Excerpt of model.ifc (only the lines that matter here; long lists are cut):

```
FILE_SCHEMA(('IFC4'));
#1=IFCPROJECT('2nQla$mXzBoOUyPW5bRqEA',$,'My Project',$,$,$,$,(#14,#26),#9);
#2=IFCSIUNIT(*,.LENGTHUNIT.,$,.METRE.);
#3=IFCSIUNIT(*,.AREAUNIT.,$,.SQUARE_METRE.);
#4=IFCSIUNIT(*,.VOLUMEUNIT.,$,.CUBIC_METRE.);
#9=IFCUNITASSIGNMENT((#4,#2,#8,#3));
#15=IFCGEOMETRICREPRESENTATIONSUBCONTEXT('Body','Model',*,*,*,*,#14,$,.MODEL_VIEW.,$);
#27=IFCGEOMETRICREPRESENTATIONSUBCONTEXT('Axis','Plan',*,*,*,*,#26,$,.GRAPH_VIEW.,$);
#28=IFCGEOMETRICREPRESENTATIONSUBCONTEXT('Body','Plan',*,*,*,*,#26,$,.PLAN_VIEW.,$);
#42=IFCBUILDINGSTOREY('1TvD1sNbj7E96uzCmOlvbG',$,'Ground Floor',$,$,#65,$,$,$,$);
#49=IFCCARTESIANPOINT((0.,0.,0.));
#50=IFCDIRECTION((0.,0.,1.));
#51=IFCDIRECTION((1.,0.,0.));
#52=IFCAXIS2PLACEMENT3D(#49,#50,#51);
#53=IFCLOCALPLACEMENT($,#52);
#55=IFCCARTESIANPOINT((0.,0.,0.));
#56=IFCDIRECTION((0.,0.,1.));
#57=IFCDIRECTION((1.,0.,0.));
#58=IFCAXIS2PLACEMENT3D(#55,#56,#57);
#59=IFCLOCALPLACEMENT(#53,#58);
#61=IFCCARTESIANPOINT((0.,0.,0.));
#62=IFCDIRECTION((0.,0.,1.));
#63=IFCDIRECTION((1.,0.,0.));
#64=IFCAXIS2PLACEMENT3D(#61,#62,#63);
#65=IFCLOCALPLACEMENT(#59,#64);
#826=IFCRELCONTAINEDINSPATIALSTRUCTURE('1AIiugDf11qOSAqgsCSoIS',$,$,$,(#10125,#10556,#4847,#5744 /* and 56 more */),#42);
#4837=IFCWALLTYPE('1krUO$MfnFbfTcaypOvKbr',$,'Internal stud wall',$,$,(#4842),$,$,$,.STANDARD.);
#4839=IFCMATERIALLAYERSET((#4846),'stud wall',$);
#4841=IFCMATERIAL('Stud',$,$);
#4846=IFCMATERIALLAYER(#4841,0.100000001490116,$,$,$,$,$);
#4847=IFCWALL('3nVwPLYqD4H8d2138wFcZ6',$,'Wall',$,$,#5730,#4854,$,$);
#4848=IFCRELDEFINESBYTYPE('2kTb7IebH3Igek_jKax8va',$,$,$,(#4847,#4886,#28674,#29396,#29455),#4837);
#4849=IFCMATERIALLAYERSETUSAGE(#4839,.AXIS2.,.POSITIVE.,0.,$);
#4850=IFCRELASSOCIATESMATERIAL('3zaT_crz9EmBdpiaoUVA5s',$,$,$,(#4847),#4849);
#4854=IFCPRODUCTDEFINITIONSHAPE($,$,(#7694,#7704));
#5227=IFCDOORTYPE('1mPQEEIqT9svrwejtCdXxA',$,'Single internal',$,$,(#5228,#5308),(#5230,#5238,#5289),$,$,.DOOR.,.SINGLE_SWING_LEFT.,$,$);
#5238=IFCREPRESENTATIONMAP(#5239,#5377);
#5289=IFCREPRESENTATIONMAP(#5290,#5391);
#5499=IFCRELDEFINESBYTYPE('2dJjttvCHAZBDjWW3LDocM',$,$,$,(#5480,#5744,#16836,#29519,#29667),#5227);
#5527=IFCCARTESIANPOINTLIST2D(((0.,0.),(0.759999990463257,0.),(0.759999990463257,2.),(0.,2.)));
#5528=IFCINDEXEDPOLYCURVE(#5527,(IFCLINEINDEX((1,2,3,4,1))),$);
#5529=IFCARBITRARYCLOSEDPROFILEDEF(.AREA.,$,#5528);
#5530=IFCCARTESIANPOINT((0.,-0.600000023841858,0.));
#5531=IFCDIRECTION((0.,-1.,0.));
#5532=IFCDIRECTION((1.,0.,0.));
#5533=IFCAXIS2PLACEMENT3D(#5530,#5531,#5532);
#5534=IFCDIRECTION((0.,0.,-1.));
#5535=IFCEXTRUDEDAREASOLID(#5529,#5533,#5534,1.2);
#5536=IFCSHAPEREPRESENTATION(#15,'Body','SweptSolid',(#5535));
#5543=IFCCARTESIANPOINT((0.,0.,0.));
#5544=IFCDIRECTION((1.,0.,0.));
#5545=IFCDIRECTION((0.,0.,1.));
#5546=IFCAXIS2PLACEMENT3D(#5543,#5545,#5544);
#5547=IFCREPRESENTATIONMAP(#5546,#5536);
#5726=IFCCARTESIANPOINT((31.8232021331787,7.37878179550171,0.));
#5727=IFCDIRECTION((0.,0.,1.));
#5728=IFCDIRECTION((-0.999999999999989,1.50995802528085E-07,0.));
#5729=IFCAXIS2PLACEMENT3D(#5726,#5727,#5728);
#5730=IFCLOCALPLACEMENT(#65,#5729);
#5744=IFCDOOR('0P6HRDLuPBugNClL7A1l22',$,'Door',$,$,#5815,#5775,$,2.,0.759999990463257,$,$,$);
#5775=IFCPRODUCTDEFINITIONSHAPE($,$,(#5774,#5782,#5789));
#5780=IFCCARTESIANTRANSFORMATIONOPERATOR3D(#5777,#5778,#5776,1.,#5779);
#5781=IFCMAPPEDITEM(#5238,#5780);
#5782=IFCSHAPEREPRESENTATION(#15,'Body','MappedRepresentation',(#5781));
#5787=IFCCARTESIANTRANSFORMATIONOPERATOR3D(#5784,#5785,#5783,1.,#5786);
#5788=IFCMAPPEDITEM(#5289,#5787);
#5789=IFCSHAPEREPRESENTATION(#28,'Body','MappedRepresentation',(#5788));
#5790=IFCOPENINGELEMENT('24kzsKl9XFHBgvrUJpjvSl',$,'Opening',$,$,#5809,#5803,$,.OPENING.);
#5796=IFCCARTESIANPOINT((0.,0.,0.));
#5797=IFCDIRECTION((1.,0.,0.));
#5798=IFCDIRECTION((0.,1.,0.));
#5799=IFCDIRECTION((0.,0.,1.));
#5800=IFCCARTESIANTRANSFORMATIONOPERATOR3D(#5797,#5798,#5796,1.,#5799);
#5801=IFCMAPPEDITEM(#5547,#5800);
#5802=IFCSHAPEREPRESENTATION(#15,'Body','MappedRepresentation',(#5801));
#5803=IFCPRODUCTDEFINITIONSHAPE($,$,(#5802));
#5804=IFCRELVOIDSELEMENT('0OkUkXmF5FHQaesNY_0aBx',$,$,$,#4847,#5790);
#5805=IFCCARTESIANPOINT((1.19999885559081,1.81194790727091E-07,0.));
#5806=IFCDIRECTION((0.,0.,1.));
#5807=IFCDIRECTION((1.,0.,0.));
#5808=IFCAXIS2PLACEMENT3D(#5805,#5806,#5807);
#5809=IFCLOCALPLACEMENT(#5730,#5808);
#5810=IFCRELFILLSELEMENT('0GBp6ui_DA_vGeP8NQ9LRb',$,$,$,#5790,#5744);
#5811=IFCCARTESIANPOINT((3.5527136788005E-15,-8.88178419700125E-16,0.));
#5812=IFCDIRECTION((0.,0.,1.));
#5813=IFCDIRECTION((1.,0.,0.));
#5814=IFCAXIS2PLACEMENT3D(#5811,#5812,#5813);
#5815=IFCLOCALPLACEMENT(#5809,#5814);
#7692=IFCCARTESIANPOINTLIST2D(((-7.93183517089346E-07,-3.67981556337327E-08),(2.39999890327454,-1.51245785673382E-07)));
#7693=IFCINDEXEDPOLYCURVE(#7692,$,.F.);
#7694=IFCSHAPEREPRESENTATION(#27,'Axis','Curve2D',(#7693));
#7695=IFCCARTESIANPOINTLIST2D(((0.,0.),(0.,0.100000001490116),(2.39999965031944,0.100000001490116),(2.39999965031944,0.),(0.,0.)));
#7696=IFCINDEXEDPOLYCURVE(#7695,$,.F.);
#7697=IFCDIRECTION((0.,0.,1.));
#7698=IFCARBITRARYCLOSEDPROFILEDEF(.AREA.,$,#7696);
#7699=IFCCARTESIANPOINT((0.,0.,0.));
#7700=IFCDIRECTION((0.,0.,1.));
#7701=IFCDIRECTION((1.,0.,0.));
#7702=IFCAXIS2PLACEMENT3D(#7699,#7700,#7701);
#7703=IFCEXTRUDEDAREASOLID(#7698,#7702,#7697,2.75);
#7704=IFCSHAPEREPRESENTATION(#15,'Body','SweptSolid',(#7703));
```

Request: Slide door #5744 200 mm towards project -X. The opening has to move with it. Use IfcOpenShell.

```python
import ifcopenshell
import ifcopenshell.api.geometry
import ifcopenshell.util.placement
import ifcopenshell.util.unit

model = ifcopenshell.open("model.ifc")
unit_scale = ifcopenshell.util.unit.calculate_unit_scale(model)

door = model.by_guid("0P6HRDLuPBugNClL7A1l22")
opening = door.FillsVoids[0].RelatingOpeningElement
wall = opening.VoidsElements[0].RelatingBuildingElement

wall_matrix = ifcopenshell.util.placement.get_local_placement(wall.ObjectPlacement)
shift = wall_matrix[:3, 0] * 0.2 / unit_scale
before = ifcopenshell.util.placement.get_local_placement(door.ObjectPlacement)[:3, 3].copy()

# The door is placed relative to its opening, so it follows when the opening moves.
matrix = ifcopenshell.util.placement.get_local_placement(opening.ObjectPlacement)
matrix[:3, 3] += shift
ifcopenshell.api.geometry.edit_object_placement(
    model, product=opening, matrix=matrix, is_si=False, should_transform_children=True
)

after = ifcopenshell.util.placement.get_local_placement(door.ObjectPlacement)[:3, 3]
print("door moved by", (after - before).round(3) + 0.0)

model.write("model-out.ifc")
```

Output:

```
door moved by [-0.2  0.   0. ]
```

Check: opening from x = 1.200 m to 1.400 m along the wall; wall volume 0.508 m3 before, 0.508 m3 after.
